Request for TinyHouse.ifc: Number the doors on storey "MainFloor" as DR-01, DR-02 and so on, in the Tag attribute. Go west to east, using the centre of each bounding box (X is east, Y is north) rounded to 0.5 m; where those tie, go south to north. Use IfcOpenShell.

First a look at what the model holds.

```python
import ifcopenshell
import ifcopenshell.util.element
import ifcopenshell.util.placement

model = ifcopenshell.open("TinyHouse.ifc")
print(model.schema)
storey = next(s for s in model.by_type("IfcBuildingStorey") if s.Name == "MainFloor")
doors = [e for e in ifcopenshell.util.element.get_decomposition(storey) if e.is_a("IfcDoor")]
for e in sorted(doors, key=lambda e: e.id()):
    origin = ifcopenshell.util.placement.get_local_placement(e.ObjectPlacement)[:3, 3]
    print(e.id(), e.Tag, e.Name, origin.round(2) + 0.0, sep=" | ")
```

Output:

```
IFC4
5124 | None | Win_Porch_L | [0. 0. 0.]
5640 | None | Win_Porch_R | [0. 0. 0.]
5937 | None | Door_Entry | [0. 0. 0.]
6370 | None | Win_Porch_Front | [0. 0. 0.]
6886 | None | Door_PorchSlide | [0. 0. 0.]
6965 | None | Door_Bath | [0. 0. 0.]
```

```python
import ifcopenshell
import ifcopenshell.geom
import ifcopenshell.util.element
import ifcopenshell.util.shape

model = ifcopenshell.open("TinyHouse.ifc")
settings = ifcopenshell.geom.settings()
settings.set("use-world-coords", True)


def centre(element):
    shape = ifcopenshell.geom.create_shape(settings, element)
    return ifcopenshell.util.shape.get_bbox_centroid(shape.geometry)


storey = next(s for s in model.by_type("IfcBuildingStorey") if s.Name == "MainFloor")
doors = [e for e in ifcopenshell.util.element.get_decomposition(storey) if e.is_a("IfcDoor")]

# Insertion points can sit at a corner or the storey origin, so sort by the geometry (in metres).
centres = {e: centre(e) for e in doors}
doors.sort(key=lambda e: (round(centres[e][0] / 0.5), centres[e][1]))

for i, e in enumerate(doors, start=1):
    number = f"DR-{i:02d}"
    e.Tag = number
    print(e.id(), number)

model.write("TinyHouse_v2.ifc")
```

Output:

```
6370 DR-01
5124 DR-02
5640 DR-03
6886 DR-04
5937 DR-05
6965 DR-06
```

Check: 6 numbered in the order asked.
